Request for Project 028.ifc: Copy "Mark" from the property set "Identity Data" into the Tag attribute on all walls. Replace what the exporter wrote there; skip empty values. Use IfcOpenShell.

First a look at what the model holds.

```python
import ifcopenshell
import ifcopenshell.util.element

model = ifcopenshell.open("Project 028.ifc")
print(model.schema)
walls = model.by_type("IfcWall")
print(len(walls), "walls")
for e in walls[:8]:
    source = ifcopenshell.util.element.get_pset(e, "Identity Data", "Mark")
    target = e.Tag
    print(e.id(), repr(source), repr(target), sep=" | ")
```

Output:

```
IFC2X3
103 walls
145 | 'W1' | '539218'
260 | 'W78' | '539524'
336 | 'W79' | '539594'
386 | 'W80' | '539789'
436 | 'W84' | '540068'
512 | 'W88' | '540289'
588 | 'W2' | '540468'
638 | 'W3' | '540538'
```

```python
import ifcopenshell
import ifcopenshell.util.element

model = ifcopenshell.open("Project 028.ifc")

count = 0
for e in model.by_type("IfcWall"):
    value = ifcopenshell.util.element.get_pset(e, "Identity Data", "Mark")
    current = e.Tag
    if not value or not value.strip() or current == value:
        continue
    e.Tag = value
    count += 1

print(count, "walls updated")

model.write("Project 028_edited.ifc")
```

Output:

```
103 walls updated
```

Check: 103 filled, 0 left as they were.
